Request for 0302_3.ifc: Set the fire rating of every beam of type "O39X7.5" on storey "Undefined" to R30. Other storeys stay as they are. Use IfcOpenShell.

First a look at what the model holds.

```python
import ifcopenshell
import ifcopenshell.util.element

model = ifcopenshell.open("0302_3.ifc")
print(model.schema)
storey = next(s for s in model.by_type("IfcBuildingStorey") if s.Name == "Undefined")
beams = [e for e in ifcopenshell.util.element.get_decomposition(storey) if e.is_a("IfcBeam")]
seen = {}
for e in beams:
    element_type = ifcopenshell.util.element.get_type(e)
    key = (element_type.Name if element_type != e and element_type else None, ifcopenshell.util.element.get_pset(e, "Pset_BeamCommon", "FireRating"))
    seen[key] = seen.get(key, 0) + 1
for (name, value), count in sorted(seen.items(), key=str):
    print(count, "x", name, "|", value)
```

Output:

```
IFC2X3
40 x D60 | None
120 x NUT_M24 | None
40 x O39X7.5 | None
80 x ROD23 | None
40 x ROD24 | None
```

```python
import ifcopenshell
import ifcopenshell.api.pset
import ifcopenshell.util.element

model = ifcopenshell.open("0302_3.ifc")

storey = next(s for s in model.by_type("IfcBuildingStorey") if s.Name == "Undefined")
beams = [e for e in ifcopenshell.util.element.get_decomposition(storey) if e.is_a("IfcBeam")]

count = 0
for e in beams:
    element_type = ifcopenshell.util.element.get_type(e)
    if element_type in (None, e) or element_type.Name != "O39X7.5":
        continue
    found = ifcopenshell.util.element.get_pset(e, "Pset_BeamCommon", should_inherit=False)
    if found:
        pset = model.by_id(found["id"])
        if len(ifcopenshell.util.element.get_elements_by_pset(pset)) > 1:
            pset = ifcopenshell.api.pset.unshare_pset(model, products=[e], pset=pset)[0]
    else:
        pset = ifcopenshell.api.pset.add_pset(model, product=e, name="Pset_BeamCommon")
    ifcopenshell.api.pset.edit_pset(model, pset=pset, properties={"FireRating": "R30"})
    count += 1

print(count, "beams updated")

model.write("0302_3_updated.ifc")
```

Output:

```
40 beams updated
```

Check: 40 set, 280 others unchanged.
